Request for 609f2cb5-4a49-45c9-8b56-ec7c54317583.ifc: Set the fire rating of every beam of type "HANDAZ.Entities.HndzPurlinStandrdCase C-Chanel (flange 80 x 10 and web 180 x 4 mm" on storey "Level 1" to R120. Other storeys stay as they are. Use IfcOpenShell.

First a look at what the model holds.

```python
import ifcopenshell
import ifcopenshell.util.element

model = ifcopenshell.open("609f2cb5-4a49-45c9-8b56-ec7c54317583.ifc")
print(model.schema)
storey = next(s for s in model.by_type("IfcBuildingStorey") if s.Name == "Level 1")
beams = [e for e in ifcopenshell.util.element.get_decomposition(storey) if e.is_a("IfcBeam")]
seen = {}
for e in beams:
    element_type = ifcopenshell.util.element.get_type(e)
    key = (element_type.Name if element_type != e and element_type else None, ifcopenshell.util.element.get_pset(e, "Pset_BeamCommon", "FireRating"))
    seen[key] = seen.get(key, 0) + 1
for (name, value), count in sorted(seen.items(), key=str):
    print(count, "x", name, "|", value)
```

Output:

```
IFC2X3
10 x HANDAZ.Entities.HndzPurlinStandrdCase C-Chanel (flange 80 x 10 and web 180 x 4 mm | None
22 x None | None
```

```python
import ifcopenshell
import ifcopenshell.api.pset
import ifcopenshell.util.element

model = ifcopenshell.open("609f2cb5-4a49-45c9-8b56-ec7c54317583.ifc")

storey = next(s for s in model.by_type("IfcBuildingStorey") if s.Name == "Level 1")
beams = [e for e in ifcopenshell.util.element.get_decomposition(storey) if e.is_a("IfcBeam")]

count = 0
for e in beams:
    element_type = ifcopenshell.util.element.get_type(e)
    if element_type in (None, e) or element_type.Name != "HANDAZ.Entities.HndzPurlinStandrdCase C-Chanel (flange 80 x 10 and web 180 x 4 mm":
        continue
    # add_pset returns the element's existing set when there is one.
    pset = ifcopenshell.api.pset.add_pset(model, product=e, name="Pset_BeamCommon")
    ifcopenshell.api.pset.edit_pset(model, pset=pset, properties={"FireRating": "R120"})
    count += 1

print(count, "beams updated")

model.write("609f2cb5-4a49-45c9-8b56-ec7c54317583_rev.ifc")
```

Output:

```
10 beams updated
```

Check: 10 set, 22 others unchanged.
